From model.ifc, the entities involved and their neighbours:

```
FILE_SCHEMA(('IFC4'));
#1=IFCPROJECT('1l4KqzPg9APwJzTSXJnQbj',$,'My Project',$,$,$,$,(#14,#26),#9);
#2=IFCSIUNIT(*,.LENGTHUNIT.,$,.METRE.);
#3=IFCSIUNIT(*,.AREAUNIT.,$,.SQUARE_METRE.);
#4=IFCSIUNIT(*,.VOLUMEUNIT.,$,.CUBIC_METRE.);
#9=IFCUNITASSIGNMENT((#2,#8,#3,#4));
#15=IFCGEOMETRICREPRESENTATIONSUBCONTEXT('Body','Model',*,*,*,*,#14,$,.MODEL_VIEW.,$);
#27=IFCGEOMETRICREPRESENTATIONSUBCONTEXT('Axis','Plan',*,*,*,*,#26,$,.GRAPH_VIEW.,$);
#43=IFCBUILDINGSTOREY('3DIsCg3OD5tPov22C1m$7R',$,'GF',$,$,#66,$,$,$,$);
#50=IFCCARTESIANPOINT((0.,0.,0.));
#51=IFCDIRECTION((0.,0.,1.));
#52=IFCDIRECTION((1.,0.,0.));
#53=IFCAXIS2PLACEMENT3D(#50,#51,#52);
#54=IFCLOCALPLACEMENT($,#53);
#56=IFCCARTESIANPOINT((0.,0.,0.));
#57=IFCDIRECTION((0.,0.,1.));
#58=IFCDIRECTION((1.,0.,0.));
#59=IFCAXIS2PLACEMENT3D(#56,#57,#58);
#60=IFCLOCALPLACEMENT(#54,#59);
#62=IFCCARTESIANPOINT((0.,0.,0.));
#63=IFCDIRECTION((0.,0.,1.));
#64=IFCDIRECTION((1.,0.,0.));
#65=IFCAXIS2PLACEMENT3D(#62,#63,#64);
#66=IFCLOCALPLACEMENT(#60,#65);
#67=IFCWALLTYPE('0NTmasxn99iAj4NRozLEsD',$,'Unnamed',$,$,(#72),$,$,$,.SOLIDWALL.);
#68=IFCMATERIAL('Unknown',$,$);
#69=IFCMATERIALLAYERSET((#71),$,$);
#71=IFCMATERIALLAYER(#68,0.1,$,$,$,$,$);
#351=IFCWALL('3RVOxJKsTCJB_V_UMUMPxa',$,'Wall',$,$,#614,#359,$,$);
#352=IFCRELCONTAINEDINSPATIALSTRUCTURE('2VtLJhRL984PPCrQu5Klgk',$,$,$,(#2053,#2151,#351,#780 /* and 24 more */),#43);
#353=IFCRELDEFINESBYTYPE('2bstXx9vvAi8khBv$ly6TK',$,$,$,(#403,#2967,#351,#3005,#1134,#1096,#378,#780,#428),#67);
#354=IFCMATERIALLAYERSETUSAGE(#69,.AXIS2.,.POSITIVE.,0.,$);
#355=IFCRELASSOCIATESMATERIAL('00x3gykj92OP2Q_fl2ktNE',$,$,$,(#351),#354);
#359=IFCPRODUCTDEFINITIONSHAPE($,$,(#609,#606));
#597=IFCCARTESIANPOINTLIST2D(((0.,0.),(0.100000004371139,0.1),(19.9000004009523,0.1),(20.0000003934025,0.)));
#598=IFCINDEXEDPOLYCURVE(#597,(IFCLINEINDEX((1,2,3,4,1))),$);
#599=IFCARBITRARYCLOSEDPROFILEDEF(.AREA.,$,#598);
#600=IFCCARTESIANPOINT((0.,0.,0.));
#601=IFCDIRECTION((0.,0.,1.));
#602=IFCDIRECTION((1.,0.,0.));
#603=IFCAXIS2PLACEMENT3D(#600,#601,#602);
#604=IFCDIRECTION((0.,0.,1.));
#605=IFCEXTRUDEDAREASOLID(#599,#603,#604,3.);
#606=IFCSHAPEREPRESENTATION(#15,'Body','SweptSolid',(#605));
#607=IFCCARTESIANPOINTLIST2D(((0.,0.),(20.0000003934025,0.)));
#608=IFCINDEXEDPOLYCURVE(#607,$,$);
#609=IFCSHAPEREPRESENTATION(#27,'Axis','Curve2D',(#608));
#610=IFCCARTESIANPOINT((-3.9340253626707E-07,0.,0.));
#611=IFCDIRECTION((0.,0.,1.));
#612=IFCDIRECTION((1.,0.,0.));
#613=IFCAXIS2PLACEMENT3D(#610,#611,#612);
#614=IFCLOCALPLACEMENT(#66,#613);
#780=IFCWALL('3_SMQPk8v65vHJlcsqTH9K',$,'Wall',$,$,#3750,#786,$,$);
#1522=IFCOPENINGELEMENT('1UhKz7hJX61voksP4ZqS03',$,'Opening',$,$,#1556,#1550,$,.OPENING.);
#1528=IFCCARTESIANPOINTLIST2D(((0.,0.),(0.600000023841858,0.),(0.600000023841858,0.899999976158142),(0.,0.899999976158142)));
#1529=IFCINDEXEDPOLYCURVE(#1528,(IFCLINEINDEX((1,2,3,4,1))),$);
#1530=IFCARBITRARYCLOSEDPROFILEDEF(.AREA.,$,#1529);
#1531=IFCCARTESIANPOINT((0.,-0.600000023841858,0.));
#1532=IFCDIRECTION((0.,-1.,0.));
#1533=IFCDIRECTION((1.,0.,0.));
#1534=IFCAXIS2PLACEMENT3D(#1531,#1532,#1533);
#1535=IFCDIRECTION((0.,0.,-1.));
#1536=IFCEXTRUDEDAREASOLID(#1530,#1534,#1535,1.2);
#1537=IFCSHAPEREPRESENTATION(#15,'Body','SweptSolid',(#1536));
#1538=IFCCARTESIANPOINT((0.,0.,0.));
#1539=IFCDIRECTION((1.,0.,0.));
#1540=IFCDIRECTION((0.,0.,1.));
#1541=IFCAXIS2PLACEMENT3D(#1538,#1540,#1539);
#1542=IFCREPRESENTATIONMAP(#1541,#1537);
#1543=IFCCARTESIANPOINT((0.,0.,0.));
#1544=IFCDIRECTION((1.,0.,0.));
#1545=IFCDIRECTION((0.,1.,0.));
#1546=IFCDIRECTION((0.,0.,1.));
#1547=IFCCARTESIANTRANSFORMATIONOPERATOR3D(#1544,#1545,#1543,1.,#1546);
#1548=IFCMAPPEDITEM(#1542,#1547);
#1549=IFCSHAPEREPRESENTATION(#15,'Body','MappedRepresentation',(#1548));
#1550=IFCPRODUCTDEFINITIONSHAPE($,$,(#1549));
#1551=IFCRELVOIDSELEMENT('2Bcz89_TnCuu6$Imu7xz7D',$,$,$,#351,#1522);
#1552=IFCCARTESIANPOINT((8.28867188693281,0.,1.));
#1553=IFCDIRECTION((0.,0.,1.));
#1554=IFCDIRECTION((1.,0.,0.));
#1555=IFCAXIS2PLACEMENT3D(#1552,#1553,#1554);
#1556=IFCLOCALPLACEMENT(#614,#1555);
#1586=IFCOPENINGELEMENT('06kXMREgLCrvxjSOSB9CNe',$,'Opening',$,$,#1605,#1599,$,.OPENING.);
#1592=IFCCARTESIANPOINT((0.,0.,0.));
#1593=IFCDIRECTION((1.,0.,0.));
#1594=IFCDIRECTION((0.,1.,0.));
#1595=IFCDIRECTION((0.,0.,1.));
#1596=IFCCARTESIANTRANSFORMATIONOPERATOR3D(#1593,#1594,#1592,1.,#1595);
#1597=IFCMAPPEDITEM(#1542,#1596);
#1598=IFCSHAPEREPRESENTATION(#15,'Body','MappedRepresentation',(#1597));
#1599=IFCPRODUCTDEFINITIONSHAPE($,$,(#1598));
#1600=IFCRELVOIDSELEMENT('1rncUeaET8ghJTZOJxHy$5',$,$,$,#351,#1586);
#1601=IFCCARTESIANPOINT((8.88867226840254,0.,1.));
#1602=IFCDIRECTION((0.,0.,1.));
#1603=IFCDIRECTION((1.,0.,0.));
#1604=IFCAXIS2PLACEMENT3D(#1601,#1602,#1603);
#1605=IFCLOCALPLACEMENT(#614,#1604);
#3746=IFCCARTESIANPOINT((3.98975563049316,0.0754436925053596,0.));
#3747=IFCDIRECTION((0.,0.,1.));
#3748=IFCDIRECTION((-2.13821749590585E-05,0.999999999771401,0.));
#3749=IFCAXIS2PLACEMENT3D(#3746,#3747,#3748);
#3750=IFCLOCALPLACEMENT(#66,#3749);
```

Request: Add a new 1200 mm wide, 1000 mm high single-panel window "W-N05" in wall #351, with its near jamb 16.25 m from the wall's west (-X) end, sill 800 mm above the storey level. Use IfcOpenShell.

```python
import numpy as np
import ifcopenshell
import ifcopenshell.api.feature
import ifcopenshell.api.geometry
import ifcopenshell.api.root
import ifcopenshell.api.spatial
import ifcopenshell.geom
import ifcopenshell.util.element
import ifcopenshell.util.placement
import ifcopenshell.util.representation
import ifcopenshell.util.shape
import ifcopenshell.util.unit

model = ifcopenshell.open("model.ifc")
unit_scale = ifcopenshell.util.unit.calculate_unit_scale(model)
settings = ifcopenshell.geom.settings()


def volume(element):
    """Net volume in cubic metres, openings subtracted."""
    shape = ifcopenshell.geom.create_shape(settings, element)
    return ifcopenshell.util.shape.get_volume(shape.geometry)


wall = model.by_id(351)
storey = ifcopenshell.util.element.get_container(wall, ifc_class="IfcBuildingStorey")
context = ifcopenshell.util.representation.get_context(model, "Model", "Body", "MODEL_VIEW")
before = volume(wall)

width, height, from_end, sill = 1.2, 1, 16.25, 0.8  # metres

# The wall runs along its own X axis, and the end named is its -X end.
wall_shape = ifcopenshell.geom.create_shape(settings, wall)
x, y, z = ifcopenshell.util.shape.get_vertices(wall_shape.geometry).T
start = x.min() + from_end
face, thickness = float(y.min()), float(y.max() - y.min())
wall_matrix = ifcopenshell.util.placement.get_local_placement(wall.ObjectPlacement)
level = ifcopenshell.util.placement.get_local_placement(storey.ObjectPlacement)[2, 3]


def in_wall(x, y):
    """Placement at x, y metres in the wall's axes, at sill height."""
    matrix = wall_matrix.copy()
    matrix[:, 3] = wall_matrix @ np.array([x / unit_scale, y / unit_scale, 0.0, 1.0])
    matrix[2, 3] = level + sill / unit_scale
    return matrix


# Opening: a box that overshoots both wall faces by 50 mm.
opening = ifcopenshell.api.root.create_entity(model, ifc_class="IfcOpeningElement", predefined_type="OPENING")
box = ifcopenshell.api.geometry.add_wall_representation(
    model, context=context, length=width, height=height, thickness=thickness + 0.1
)
ifcopenshell.api.geometry.assign_representation(model, product=opening, representation=box)
ifcopenshell.api.geometry.edit_object_placement(model, product=opening, matrix=in_wall(start, face - 0.05), is_si=False)
ifcopenshell.api.feature.add_feature(model, feature=opening, element=wall)

window = ifcopenshell.api.root.create_entity(model, ifc_class="IfcWindow", name="W-N05", predefined_type="WINDOW")
window.OverallWidth, window.OverallHeight = width / unit_scale, height / unit_scale
window.PartitioningType = "SINGLE_PANEL"
body = ifcopenshell.api.geometry.add_window_representation(
    model,
    context=context,
    overall_width=window.OverallWidth,
    overall_height=window.OverallHeight,
    partition_type="SINGLE_PANEL",
)
ifcopenshell.api.geometry.assign_representation(model, product=window, representation=body)
ifcopenshell.api.spatial.assign_container(model, products=[window], relating_structure=storey)
ifcopenshell.api.feature.add_filling(model, opening=opening, element=window)

# Centre the window in the wall's thickness.
ifcopenshell.api.geometry.edit_object_placement(model, product=window, matrix=in_wall(start, face), is_si=False)
window_shape = ifcopenshell.geom.create_shape(settings, window)
depth = ifcopenshell.util.shape.get_vertices(window_shape.geometry)[:, 1]
offset = face + thickness / 2 - (depth.min() + depth.max()) / 2
ifcopenshell.api.geometry.edit_object_placement(model, product=window, matrix=in_wall(start, offset), is_si=False)

after = volume(wall)

print(f"wall volume {before:.3f} -> {after:.3f} m3")

model.write("model_v2.ifc")
```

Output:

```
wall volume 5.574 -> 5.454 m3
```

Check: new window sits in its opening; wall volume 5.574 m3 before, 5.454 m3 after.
